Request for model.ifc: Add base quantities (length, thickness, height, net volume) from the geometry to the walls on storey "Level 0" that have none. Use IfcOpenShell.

First a look at what the model holds.

```python
import ifcopenshell
import ifcopenshell.util.element
import ifcopenshell.util.unit

model = ifcopenshell.open("model.ifc")
print(model.schema)
for unit_type in ("LENGTHUNIT", "AREAUNIT", "VOLUMEUNIT"):
    print(unit_type, ifcopenshell.util.unit.calculate_unit_scale(model, unit_type))
storey = next(s for s in model.by_type("IfcBuildingStorey") if s.Name == "Level 0")
walls = [e for e in ifcopenshell.util.element.get_decomposition(storey) if e.is_a("IfcWall")]
for e in sorted(walls, key=lambda e: e.id()):
    print(e.id(), e.is_a(), e.Name, list(ifcopenshell.util.element.get_psets(e, qtos_only=True)), sep=" | ")
```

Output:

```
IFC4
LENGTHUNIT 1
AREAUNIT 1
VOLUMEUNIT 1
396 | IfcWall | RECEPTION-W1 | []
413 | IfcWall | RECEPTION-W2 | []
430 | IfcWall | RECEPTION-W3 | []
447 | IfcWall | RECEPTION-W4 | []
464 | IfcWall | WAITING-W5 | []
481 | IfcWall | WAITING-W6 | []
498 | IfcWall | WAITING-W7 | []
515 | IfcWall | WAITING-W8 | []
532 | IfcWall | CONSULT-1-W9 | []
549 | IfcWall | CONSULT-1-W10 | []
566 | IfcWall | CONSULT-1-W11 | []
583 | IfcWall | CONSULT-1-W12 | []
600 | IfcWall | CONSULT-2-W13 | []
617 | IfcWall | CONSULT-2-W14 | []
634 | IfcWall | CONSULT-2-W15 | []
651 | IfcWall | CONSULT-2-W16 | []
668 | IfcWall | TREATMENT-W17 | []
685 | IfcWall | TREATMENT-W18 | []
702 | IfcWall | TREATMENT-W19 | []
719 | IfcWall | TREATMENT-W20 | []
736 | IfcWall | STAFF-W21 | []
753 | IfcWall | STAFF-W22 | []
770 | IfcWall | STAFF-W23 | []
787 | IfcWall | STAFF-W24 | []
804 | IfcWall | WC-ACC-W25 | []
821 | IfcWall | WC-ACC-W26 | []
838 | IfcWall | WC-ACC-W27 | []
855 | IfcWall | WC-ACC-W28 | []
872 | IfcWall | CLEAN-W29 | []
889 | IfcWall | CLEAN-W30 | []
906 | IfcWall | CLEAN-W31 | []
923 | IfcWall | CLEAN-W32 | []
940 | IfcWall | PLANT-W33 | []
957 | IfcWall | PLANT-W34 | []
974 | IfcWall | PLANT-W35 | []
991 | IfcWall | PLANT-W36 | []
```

```python
import ifcopenshell
import ifcopenshell.api.pset
import ifcopenshell.geom
import ifcopenshell.util.element
import ifcopenshell.util.shape
import ifcopenshell.util.unit

model = ifcopenshell.open("model.ifc")
unit_scale = ifcopenshell.util.unit.calculate_unit_scale(model)
volume_scale = ifcopenshell.util.unit.calculate_unit_scale(model, "VOLUMEUNIT")
settings = ifcopenshell.geom.settings()

storey = next(s for s in model.by_type("IfcBuildingStorey") if s.Name == "Level 0")
walls = [e for e in ifcopenshell.util.element.get_decomposition(storey) if e.is_a("IfcWall")]

for e in sorted(walls, key=lambda e: e.id()):
    if ifcopenshell.util.element.get_psets(e, qtos_only=True, should_inherit=False):
        continue
    # Geometry comes back in metres, in the element's own axes.
    shape = ifcopenshell.geom.create_shape(settings, e)
    values = {
        "Length": ifcopenshell.util.shape.get_x(shape.geometry) / unit_scale,
        "Width": ifcopenshell.util.shape.get_y(shape.geometry) / unit_scale,
        "Height": ifcopenshell.util.shape.get_z(shape.geometry) / unit_scale,
        "NetVolume": ifcopenshell.util.shape.get_volume(shape.geometry) / volume_scale,
    }
    qto = ifcopenshell.api.pset.add_qto(model, product=e, name="Qto_WallBaseQuantities")
    ifcopenshell.api.pset.edit_qto(model, qto=qto, properties=values)
    print(e.id(), {k: round(v, 3) for k, v in values.items()})

model.write("model_updated.ifc")
```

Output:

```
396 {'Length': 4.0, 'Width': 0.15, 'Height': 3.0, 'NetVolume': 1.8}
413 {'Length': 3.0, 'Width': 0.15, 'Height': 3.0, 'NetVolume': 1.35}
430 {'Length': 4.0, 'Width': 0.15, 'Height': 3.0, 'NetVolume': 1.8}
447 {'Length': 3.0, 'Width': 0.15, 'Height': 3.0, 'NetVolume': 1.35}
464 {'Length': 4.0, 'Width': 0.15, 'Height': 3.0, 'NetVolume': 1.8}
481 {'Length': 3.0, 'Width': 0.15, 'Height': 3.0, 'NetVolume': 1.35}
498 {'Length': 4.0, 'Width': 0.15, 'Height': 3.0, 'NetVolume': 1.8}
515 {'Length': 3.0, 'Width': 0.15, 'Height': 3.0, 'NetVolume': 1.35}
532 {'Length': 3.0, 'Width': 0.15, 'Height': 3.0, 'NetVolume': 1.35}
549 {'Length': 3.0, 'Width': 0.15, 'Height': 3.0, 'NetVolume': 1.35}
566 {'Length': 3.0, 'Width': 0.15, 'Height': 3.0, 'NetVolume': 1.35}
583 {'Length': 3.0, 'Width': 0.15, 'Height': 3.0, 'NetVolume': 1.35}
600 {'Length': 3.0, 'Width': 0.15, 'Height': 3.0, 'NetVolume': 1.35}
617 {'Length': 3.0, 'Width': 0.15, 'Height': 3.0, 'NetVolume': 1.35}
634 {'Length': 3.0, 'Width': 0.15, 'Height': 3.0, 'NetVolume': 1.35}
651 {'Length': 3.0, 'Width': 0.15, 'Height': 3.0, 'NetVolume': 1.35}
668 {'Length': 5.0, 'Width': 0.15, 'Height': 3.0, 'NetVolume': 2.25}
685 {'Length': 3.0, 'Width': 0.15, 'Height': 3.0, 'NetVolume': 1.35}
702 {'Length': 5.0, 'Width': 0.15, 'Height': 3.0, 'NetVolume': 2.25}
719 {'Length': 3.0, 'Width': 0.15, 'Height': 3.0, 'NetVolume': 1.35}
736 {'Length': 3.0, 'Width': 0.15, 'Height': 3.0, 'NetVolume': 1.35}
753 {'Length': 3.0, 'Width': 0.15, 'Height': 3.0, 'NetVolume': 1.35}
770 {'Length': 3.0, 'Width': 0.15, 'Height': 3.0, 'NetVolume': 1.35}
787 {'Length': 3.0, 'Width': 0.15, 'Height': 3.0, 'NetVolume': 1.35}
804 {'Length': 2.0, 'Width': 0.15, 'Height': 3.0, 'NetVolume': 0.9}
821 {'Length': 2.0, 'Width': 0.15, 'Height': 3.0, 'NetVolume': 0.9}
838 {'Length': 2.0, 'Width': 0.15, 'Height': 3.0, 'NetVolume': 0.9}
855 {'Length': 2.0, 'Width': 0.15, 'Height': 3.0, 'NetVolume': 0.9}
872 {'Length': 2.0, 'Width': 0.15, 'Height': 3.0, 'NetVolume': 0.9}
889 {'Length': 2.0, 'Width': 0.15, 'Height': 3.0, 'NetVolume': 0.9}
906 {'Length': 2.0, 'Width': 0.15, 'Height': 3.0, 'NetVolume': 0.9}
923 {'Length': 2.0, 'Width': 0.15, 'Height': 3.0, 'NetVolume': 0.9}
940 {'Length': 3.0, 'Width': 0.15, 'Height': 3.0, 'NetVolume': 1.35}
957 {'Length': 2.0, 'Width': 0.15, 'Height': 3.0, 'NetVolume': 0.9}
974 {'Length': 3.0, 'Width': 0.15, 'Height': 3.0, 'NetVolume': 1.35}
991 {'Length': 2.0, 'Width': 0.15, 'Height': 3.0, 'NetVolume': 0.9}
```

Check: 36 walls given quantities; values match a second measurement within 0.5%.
